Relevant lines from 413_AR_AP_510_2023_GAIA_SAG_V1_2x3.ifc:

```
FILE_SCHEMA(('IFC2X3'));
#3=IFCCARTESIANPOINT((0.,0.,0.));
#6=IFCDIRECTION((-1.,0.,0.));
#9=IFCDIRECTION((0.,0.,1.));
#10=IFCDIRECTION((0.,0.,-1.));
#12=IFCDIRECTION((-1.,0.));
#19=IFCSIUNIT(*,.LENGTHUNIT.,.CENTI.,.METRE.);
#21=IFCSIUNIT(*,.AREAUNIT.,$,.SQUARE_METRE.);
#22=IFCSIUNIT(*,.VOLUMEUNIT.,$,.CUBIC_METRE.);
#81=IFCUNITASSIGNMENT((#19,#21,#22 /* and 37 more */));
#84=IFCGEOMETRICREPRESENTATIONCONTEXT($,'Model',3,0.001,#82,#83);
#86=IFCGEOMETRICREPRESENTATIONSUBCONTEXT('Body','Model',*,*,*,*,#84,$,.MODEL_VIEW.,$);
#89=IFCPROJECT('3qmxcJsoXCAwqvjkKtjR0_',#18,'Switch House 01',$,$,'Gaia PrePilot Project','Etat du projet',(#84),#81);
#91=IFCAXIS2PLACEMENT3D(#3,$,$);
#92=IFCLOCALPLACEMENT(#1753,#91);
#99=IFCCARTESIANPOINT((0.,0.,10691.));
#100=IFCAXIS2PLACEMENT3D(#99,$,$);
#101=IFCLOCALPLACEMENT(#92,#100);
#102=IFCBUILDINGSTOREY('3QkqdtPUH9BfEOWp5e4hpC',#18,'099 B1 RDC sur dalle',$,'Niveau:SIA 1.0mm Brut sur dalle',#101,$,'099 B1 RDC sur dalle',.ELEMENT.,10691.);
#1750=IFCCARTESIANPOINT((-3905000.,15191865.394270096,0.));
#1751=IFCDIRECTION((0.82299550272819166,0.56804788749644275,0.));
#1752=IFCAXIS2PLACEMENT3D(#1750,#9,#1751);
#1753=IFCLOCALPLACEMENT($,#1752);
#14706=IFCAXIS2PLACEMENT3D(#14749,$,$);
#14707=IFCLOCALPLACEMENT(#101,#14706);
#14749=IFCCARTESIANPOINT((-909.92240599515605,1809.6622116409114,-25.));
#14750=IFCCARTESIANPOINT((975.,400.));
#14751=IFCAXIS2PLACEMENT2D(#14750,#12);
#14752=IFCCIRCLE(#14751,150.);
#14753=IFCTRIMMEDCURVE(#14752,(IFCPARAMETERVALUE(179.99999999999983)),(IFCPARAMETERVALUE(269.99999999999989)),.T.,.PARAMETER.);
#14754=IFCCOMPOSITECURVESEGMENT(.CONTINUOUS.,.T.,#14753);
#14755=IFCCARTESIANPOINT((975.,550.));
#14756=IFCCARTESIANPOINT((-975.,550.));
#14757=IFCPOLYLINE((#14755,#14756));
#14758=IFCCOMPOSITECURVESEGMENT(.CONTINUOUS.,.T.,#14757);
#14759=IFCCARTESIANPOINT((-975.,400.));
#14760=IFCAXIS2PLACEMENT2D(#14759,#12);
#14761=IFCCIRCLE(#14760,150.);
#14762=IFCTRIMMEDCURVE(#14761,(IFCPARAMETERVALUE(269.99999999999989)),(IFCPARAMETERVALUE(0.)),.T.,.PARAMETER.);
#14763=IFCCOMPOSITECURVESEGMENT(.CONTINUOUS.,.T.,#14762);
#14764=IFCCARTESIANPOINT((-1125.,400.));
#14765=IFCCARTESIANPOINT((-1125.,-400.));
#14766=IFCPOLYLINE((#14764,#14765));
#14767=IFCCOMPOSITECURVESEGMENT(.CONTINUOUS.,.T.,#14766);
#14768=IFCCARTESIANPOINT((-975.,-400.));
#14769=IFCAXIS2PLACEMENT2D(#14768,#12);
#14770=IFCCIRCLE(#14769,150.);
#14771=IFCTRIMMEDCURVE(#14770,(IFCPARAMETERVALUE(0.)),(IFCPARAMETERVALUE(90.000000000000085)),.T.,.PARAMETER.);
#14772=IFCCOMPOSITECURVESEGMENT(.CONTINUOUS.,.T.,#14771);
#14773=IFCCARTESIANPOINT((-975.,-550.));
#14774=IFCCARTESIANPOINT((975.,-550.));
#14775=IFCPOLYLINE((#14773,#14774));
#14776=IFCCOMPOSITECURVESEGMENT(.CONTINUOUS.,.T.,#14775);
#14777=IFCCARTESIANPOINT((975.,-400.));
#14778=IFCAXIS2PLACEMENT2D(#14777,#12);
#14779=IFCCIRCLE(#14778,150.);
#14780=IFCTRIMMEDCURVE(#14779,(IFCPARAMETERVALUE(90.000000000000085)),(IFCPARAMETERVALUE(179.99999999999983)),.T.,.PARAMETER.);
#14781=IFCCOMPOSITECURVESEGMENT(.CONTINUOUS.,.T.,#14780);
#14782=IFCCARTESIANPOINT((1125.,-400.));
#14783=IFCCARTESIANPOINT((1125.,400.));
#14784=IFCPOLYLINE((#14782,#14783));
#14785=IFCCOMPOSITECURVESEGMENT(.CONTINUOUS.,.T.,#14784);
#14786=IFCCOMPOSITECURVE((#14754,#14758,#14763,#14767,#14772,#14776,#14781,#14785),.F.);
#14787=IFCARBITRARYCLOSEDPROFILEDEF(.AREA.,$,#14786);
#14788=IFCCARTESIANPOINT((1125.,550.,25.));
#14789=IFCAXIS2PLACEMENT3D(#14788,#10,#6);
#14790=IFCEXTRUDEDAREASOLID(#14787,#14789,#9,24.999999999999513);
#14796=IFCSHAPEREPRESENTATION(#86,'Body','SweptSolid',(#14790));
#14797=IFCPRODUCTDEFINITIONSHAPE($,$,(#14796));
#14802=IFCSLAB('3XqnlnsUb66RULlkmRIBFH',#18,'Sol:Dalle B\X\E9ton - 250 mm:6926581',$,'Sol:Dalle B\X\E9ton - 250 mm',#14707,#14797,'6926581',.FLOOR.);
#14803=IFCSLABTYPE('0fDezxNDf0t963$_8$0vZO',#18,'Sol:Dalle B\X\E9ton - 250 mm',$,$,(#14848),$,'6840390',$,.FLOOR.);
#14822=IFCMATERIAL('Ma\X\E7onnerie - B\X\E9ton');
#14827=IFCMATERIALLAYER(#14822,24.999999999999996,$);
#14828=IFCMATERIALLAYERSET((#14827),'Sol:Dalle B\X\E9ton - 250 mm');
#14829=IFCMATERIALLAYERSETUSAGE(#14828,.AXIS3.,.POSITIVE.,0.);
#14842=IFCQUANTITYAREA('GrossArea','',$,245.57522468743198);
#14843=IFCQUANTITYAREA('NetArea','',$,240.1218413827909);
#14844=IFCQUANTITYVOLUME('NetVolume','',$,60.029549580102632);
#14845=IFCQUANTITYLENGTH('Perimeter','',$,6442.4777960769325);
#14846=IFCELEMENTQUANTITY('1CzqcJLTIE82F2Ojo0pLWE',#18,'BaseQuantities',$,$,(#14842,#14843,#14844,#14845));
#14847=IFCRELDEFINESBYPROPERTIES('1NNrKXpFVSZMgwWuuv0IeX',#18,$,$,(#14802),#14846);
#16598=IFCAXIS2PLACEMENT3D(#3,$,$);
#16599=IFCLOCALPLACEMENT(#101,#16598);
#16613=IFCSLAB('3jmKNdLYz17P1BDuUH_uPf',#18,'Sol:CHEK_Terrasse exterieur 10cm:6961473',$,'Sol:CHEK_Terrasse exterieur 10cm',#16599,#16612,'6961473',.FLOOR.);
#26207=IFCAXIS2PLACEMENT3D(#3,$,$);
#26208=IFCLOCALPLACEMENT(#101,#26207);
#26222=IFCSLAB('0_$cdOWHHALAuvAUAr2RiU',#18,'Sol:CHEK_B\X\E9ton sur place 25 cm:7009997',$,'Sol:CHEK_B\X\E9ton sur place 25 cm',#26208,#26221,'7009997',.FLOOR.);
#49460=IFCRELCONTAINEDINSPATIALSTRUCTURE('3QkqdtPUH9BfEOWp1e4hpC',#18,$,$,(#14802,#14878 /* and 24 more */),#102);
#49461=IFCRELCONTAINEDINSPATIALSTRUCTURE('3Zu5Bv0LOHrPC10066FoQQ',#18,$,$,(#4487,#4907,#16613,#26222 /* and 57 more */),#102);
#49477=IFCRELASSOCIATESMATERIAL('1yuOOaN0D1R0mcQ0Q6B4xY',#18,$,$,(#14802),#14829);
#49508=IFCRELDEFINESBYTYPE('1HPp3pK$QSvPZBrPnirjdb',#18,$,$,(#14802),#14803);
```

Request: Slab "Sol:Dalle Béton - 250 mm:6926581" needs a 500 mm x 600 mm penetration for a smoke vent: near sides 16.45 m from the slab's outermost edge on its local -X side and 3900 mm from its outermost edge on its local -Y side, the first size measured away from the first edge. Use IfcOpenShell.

```python
import numpy as np
import ifcopenshell
import ifcopenshell.api.feature
import ifcopenshell.api.geometry
import ifcopenshell.api.pset
import ifcopenshell.api.root
import ifcopenshell.geom
import ifcopenshell.util.element
import ifcopenshell.util.placement
import ifcopenshell.util.representation
import ifcopenshell.util.shape
import ifcopenshell.util.unit

model = ifcopenshell.open("413_AR_AP_510_2023_GAIA_SAG_V1_2x3.ifc")
unit_scale = ifcopenshell.util.unit.calculate_unit_scale(model)
area_scale = ifcopenshell.util.unit.calculate_unit_scale(model, "AREAUNIT")
volume_scale = ifcopenshell.util.unit.calculate_unit_scale(model, "VOLUMEUNIT")
settings = ifcopenshell.geom.settings()


def volume(element):
    """Net volume in cubic metres, openings subtracted."""
    shape = ifcopenshell.geom.create_shape(settings, element)
    return ifcopenshell.util.shape.get_volume(shape.geometry)


slab = model.by_guid("3XqnlnsUb66RULlkmRIBFH")
before = volume(slab)

# Extent in the slab's own axes, in metres. The edges named are its -X and -Y sides.
slab_shape = ifcopenshell.geom.create_shape(settings, slab)
vertices = ifcopenshell.util.shape.get_vertices(slab_shape.geometry)
x_min, y_min, bottom = vertices.min(axis=0)
top = vertices[:, 2].max()

opening = ifcopenshell.api.root.create_entity(model, ifc_class="IfcOpeningElement", name="Smoke vent opening")
context = ifcopenshell.util.representation.get_context(model, "Model", "Body", "MODEL_VIEW")
width, depth = 0.5, 0.6
outline = [(0.0, 0.0), (width, 0.0), (width, depth), (0.0, depth), (0.0, 0.0)]
# Overshoot both faces by 50 mm so the cut is clean.
shape = ifcopenshell.api.geometry.add_slab_representation(
    model, context=context, depth=top - bottom + 0.1, polyline=outline
)
ifcopenshell.api.geometry.assign_representation(model, product=opening, representation=shape)

matrix = ifcopenshell.util.placement.get_local_placement(slab.ObjectPlacement)
matrix[:, 3] = matrix @ np.append(np.array([x_min + 16.45, y_min + 3.9, bottom - 0.05]) / unit_scale, 1.0)
ifcopenshell.api.geometry.edit_object_placement(model, product=opening, matrix=matrix, is_si=False)
ifcopenshell.api.feature.add_feature(model, feature=opening, element=slab)

after = volume(slab)

# Update the slab's stored quantities.
qto = model.by_id(ifcopenshell.util.element.get_pset(slab, "BaseQuantities", should_inherit=False)["id"])
ifcopenshell.api.pset.edit_qto(model, qto=qto, properties={
    "NetArea": after / (top - bottom) / area_scale,
    "NetVolume": after / volume_scale,
})

print(f"slab volume {before:.3f} -> {after:.3f} m3")

model.write("413_AR_AP_510_2023_GAIA_SAG_V1_2x3_edited.ifc")
```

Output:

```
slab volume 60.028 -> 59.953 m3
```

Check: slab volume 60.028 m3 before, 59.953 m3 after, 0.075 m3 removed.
